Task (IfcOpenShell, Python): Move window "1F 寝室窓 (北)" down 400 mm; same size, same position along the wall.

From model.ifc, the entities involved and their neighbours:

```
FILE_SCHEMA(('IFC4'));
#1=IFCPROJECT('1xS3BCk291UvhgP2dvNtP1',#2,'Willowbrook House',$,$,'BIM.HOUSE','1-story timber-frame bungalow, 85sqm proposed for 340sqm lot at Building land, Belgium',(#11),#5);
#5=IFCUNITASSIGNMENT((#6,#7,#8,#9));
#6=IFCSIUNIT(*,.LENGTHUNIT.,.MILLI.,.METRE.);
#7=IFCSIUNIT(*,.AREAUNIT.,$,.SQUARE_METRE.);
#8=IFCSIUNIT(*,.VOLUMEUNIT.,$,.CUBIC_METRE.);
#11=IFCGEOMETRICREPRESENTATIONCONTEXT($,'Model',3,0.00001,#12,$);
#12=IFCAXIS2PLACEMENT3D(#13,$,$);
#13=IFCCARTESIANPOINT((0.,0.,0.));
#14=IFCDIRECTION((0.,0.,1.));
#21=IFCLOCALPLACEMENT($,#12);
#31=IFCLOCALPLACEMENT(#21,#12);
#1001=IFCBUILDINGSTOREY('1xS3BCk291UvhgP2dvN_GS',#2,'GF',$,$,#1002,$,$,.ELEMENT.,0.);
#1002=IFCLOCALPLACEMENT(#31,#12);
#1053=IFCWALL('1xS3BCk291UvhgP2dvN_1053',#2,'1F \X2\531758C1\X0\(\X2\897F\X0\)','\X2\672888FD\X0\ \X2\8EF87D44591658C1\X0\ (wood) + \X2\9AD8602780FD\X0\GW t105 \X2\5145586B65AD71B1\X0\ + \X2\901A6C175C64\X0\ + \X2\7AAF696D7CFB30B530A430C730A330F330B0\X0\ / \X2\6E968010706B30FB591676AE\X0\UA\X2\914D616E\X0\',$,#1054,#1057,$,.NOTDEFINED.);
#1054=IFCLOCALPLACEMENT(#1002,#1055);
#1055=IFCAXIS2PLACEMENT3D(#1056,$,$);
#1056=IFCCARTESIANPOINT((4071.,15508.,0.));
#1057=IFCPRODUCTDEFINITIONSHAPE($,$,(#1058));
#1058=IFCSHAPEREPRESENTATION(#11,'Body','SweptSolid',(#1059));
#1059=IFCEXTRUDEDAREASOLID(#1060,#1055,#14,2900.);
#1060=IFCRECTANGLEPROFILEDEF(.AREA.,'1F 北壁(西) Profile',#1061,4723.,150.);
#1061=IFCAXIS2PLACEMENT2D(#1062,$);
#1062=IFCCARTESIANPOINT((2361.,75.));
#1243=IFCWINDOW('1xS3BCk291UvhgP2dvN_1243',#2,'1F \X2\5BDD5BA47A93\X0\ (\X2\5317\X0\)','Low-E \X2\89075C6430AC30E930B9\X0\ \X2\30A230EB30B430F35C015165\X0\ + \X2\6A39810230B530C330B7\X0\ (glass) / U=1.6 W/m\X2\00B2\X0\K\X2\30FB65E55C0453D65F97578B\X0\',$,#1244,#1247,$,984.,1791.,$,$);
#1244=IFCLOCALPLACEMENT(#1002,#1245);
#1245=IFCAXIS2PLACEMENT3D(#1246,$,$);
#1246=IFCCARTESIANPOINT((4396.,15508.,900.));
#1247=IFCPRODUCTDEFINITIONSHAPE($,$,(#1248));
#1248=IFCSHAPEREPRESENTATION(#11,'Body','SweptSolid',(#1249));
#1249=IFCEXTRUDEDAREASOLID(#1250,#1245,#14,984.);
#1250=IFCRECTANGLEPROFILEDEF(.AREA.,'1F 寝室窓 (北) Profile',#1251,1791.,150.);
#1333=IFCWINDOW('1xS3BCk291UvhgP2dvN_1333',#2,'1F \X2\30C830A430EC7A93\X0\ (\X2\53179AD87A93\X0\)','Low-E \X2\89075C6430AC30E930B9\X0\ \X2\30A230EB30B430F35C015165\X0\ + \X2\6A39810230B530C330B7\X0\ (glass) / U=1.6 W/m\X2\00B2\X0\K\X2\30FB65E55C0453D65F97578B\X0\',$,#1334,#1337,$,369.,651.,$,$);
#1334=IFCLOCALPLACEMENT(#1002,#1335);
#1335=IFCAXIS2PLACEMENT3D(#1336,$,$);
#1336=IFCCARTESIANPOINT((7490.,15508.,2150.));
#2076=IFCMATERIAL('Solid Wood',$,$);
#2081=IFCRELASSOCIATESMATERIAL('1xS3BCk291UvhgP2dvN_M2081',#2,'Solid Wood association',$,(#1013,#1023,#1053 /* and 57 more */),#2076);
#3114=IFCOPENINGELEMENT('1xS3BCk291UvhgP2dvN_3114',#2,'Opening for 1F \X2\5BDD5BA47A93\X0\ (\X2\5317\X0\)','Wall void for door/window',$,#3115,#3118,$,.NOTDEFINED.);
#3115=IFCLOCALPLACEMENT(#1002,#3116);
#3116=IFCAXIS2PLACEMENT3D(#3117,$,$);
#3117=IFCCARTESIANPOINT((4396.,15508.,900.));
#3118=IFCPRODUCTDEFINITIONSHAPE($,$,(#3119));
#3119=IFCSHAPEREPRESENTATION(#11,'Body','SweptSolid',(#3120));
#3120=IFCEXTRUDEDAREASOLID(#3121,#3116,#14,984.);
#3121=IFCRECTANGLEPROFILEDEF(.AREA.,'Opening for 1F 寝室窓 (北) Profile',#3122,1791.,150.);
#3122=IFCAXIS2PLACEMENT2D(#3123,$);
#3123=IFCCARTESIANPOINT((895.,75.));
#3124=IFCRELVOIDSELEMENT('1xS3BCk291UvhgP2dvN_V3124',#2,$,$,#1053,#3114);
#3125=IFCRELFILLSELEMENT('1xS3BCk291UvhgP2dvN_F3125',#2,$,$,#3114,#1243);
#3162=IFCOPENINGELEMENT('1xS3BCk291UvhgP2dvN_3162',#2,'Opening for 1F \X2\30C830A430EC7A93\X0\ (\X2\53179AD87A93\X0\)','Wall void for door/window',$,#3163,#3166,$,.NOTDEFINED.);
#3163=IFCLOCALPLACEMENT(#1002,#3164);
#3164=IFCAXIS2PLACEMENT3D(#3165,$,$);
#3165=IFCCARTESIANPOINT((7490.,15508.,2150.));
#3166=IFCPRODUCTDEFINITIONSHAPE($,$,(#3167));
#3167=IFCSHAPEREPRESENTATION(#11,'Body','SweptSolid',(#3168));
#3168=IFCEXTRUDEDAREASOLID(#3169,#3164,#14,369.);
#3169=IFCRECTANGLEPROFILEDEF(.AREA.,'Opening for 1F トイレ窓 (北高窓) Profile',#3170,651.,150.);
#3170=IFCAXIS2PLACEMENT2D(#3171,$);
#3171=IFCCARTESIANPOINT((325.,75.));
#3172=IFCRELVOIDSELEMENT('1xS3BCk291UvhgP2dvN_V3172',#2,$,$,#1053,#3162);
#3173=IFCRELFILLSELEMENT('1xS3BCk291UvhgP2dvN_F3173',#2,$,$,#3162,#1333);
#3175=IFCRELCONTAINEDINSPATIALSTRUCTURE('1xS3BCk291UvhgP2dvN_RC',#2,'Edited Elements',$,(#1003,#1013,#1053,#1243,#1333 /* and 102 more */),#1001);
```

```python
import numpy as np
import ifcopenshell
import ifcopenshell.api.geometry
import ifcopenshell.util.placement
import ifcopenshell.util.unit

model = ifcopenshell.open("model.ifc")
unit_scale = ifcopenshell.util.unit.calculate_unit_scale(model)

window = model.by_id(1243)
opening = window.FillsVoids[0].RelatingOpeningElement
dz = -0.4 / unit_scale

shift = np.array([0.0, 0.0, dz])
# The window is not placed relative to its opening, so move both.
for product in (opening, window):
    matrix = ifcopenshell.util.placement.get_local_placement(product.ObjectPlacement)
    matrix[:3, 3] += shift
    ifcopenshell.api.geometry.edit_object_placement(model, product=product, matrix=matrix, is_si=False)

print(f"moved by {dz * unit_scale:+.3f} m")

model.write("model_edited.ifc")
```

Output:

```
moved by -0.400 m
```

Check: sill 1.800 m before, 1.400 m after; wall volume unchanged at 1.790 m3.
